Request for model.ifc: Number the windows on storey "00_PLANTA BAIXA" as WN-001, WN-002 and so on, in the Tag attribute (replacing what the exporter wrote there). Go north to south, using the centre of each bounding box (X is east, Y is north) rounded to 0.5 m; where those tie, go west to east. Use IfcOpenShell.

First a look at what the model holds.

```python
import ifcopenshell
import ifcopenshell.util.element
import ifcopenshell.util.placement

model = ifcopenshell.open("model.ifc")
print(model.schema)
storey = next(s for s in model.by_type("IfcBuildingStorey") if s.Name == "00_PLANTA BAIXA")
windows = [e for e in ifcopenshell.util.element.get_decomposition(storey) if e.is_a("IfcWindow")]
for e in sorted(windows, key=lambda e: e.id()):
    origin = ifcopenshell.util.placement.get_local_placement(e.ObjectPlacement)[:3, 3]
    print(e.id(), e.Tag, e.Name, origin.round(2) + 0.0, sep=" | ")
```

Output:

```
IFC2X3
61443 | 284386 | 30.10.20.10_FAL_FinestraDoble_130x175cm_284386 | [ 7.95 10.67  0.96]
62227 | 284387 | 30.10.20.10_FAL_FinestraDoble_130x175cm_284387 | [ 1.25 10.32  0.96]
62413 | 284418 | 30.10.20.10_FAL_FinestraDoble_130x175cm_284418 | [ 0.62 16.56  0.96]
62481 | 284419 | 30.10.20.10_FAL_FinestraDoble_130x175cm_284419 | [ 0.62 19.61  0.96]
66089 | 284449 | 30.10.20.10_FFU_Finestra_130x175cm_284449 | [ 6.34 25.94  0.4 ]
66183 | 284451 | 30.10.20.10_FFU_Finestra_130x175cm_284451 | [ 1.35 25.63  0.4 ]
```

```python
import ifcopenshell
import ifcopenshell.geom
import ifcopenshell.util.element
import ifcopenshell.util.shape

model = ifcopenshell.open("model.ifc")
settings = ifcopenshell.geom.settings()
settings.set("use-world-coords", True)


def centre(element):
    shape = ifcopenshell.geom.create_shape(settings, element)
    return ifcopenshell.util.shape.get_bbox_centroid(shape.geometry)


storey = next(s for s in model.by_type("IfcBuildingStorey") if s.Name == "00_PLANTA BAIXA")
windows = [e for e in ifcopenshell.util.element.get_decomposition(storey) if e.is_a("IfcWindow")]

# Insertion points can sit at a corner or the storey origin, so sort by the geometry (in metres).
centres = {e: centre(e) for e in windows}
windows.sort(key=lambda e: (-round(centres[e][1] / 0.5), centres[e][0]))

for i, e in enumerate(windows, start=1):
    number = f"WN-0{i:02d}"
    e.Tag = number
    print(e.id(), number)

model.write("model_v2.ifc")
```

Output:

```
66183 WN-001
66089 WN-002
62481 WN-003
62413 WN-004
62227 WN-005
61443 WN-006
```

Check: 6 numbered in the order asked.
